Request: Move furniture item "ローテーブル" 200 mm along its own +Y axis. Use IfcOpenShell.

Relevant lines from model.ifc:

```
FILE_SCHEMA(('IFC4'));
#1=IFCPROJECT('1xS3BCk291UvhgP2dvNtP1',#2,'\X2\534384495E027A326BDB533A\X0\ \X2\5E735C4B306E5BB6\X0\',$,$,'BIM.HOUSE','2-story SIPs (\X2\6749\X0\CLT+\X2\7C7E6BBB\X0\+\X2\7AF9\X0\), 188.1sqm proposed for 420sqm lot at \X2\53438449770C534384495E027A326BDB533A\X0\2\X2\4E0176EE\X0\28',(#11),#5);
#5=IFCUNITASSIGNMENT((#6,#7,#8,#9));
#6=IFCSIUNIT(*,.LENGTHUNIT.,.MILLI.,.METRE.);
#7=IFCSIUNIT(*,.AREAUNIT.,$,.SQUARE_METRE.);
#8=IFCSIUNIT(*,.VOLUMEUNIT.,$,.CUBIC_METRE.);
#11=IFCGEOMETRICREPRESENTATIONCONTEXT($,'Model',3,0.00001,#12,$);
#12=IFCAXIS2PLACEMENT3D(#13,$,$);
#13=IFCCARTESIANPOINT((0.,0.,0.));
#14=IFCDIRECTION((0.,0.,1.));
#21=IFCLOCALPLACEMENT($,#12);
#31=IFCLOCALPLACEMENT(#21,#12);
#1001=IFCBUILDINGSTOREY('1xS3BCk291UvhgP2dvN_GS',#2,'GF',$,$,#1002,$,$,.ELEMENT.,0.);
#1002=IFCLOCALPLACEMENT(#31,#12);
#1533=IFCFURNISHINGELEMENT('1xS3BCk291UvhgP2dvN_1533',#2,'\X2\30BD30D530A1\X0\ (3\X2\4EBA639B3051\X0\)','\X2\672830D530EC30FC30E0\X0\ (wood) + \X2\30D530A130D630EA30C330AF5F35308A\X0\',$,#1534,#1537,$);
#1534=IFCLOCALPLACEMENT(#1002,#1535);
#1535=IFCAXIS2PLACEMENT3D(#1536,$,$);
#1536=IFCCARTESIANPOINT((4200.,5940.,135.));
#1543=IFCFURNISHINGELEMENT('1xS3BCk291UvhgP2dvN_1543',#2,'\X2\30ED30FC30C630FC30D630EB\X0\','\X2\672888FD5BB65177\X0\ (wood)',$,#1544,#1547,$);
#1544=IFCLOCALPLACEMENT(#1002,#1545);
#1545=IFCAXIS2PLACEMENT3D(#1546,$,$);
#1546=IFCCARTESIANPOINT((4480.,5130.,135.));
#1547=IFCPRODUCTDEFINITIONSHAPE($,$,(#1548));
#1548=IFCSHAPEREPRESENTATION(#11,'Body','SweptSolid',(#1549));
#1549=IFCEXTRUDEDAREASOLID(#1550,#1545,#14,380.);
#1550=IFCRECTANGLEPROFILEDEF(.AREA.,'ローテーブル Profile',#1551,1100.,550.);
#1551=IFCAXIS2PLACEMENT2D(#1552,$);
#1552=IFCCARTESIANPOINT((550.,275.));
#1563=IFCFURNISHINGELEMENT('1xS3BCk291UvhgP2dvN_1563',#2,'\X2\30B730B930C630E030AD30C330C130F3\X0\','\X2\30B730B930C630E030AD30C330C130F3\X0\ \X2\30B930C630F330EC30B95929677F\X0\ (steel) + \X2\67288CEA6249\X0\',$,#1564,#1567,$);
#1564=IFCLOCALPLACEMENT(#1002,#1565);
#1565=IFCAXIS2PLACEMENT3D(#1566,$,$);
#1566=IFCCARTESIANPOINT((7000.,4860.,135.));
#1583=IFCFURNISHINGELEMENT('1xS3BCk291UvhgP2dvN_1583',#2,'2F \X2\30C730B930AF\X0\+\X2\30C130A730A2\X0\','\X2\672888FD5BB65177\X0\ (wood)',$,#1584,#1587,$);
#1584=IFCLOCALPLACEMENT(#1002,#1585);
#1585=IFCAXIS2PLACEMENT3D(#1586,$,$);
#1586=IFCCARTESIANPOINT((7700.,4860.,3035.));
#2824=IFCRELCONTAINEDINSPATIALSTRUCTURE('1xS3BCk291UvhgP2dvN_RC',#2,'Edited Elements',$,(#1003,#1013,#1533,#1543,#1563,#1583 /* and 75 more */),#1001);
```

```python
import ifcopenshell
import ifcopenshell.api.geometry
import ifcopenshell.util.placement

model = ifcopenshell.open("model.ifc")

item = model.by_guid("1xS3BCk291UvhgP2dvN_1543")
matrix = ifcopenshell.util.placement.get_local_placement(item.ObjectPlacement)
matrix[:3, 3] += matrix[:3, 1] * 200.0
ifcopenshell.api.geometry.edit_object_placement(model, product=item, matrix=matrix, is_si=False)

print(ifcopenshell.util.placement.get_local_placement(item.ObjectPlacement).round(3) + 0.0)

model.write("model_updated.ifc")
```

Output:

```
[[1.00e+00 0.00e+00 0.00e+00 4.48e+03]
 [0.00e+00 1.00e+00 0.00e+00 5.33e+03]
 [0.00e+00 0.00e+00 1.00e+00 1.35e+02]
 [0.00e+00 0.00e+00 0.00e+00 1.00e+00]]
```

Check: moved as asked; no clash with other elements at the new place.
